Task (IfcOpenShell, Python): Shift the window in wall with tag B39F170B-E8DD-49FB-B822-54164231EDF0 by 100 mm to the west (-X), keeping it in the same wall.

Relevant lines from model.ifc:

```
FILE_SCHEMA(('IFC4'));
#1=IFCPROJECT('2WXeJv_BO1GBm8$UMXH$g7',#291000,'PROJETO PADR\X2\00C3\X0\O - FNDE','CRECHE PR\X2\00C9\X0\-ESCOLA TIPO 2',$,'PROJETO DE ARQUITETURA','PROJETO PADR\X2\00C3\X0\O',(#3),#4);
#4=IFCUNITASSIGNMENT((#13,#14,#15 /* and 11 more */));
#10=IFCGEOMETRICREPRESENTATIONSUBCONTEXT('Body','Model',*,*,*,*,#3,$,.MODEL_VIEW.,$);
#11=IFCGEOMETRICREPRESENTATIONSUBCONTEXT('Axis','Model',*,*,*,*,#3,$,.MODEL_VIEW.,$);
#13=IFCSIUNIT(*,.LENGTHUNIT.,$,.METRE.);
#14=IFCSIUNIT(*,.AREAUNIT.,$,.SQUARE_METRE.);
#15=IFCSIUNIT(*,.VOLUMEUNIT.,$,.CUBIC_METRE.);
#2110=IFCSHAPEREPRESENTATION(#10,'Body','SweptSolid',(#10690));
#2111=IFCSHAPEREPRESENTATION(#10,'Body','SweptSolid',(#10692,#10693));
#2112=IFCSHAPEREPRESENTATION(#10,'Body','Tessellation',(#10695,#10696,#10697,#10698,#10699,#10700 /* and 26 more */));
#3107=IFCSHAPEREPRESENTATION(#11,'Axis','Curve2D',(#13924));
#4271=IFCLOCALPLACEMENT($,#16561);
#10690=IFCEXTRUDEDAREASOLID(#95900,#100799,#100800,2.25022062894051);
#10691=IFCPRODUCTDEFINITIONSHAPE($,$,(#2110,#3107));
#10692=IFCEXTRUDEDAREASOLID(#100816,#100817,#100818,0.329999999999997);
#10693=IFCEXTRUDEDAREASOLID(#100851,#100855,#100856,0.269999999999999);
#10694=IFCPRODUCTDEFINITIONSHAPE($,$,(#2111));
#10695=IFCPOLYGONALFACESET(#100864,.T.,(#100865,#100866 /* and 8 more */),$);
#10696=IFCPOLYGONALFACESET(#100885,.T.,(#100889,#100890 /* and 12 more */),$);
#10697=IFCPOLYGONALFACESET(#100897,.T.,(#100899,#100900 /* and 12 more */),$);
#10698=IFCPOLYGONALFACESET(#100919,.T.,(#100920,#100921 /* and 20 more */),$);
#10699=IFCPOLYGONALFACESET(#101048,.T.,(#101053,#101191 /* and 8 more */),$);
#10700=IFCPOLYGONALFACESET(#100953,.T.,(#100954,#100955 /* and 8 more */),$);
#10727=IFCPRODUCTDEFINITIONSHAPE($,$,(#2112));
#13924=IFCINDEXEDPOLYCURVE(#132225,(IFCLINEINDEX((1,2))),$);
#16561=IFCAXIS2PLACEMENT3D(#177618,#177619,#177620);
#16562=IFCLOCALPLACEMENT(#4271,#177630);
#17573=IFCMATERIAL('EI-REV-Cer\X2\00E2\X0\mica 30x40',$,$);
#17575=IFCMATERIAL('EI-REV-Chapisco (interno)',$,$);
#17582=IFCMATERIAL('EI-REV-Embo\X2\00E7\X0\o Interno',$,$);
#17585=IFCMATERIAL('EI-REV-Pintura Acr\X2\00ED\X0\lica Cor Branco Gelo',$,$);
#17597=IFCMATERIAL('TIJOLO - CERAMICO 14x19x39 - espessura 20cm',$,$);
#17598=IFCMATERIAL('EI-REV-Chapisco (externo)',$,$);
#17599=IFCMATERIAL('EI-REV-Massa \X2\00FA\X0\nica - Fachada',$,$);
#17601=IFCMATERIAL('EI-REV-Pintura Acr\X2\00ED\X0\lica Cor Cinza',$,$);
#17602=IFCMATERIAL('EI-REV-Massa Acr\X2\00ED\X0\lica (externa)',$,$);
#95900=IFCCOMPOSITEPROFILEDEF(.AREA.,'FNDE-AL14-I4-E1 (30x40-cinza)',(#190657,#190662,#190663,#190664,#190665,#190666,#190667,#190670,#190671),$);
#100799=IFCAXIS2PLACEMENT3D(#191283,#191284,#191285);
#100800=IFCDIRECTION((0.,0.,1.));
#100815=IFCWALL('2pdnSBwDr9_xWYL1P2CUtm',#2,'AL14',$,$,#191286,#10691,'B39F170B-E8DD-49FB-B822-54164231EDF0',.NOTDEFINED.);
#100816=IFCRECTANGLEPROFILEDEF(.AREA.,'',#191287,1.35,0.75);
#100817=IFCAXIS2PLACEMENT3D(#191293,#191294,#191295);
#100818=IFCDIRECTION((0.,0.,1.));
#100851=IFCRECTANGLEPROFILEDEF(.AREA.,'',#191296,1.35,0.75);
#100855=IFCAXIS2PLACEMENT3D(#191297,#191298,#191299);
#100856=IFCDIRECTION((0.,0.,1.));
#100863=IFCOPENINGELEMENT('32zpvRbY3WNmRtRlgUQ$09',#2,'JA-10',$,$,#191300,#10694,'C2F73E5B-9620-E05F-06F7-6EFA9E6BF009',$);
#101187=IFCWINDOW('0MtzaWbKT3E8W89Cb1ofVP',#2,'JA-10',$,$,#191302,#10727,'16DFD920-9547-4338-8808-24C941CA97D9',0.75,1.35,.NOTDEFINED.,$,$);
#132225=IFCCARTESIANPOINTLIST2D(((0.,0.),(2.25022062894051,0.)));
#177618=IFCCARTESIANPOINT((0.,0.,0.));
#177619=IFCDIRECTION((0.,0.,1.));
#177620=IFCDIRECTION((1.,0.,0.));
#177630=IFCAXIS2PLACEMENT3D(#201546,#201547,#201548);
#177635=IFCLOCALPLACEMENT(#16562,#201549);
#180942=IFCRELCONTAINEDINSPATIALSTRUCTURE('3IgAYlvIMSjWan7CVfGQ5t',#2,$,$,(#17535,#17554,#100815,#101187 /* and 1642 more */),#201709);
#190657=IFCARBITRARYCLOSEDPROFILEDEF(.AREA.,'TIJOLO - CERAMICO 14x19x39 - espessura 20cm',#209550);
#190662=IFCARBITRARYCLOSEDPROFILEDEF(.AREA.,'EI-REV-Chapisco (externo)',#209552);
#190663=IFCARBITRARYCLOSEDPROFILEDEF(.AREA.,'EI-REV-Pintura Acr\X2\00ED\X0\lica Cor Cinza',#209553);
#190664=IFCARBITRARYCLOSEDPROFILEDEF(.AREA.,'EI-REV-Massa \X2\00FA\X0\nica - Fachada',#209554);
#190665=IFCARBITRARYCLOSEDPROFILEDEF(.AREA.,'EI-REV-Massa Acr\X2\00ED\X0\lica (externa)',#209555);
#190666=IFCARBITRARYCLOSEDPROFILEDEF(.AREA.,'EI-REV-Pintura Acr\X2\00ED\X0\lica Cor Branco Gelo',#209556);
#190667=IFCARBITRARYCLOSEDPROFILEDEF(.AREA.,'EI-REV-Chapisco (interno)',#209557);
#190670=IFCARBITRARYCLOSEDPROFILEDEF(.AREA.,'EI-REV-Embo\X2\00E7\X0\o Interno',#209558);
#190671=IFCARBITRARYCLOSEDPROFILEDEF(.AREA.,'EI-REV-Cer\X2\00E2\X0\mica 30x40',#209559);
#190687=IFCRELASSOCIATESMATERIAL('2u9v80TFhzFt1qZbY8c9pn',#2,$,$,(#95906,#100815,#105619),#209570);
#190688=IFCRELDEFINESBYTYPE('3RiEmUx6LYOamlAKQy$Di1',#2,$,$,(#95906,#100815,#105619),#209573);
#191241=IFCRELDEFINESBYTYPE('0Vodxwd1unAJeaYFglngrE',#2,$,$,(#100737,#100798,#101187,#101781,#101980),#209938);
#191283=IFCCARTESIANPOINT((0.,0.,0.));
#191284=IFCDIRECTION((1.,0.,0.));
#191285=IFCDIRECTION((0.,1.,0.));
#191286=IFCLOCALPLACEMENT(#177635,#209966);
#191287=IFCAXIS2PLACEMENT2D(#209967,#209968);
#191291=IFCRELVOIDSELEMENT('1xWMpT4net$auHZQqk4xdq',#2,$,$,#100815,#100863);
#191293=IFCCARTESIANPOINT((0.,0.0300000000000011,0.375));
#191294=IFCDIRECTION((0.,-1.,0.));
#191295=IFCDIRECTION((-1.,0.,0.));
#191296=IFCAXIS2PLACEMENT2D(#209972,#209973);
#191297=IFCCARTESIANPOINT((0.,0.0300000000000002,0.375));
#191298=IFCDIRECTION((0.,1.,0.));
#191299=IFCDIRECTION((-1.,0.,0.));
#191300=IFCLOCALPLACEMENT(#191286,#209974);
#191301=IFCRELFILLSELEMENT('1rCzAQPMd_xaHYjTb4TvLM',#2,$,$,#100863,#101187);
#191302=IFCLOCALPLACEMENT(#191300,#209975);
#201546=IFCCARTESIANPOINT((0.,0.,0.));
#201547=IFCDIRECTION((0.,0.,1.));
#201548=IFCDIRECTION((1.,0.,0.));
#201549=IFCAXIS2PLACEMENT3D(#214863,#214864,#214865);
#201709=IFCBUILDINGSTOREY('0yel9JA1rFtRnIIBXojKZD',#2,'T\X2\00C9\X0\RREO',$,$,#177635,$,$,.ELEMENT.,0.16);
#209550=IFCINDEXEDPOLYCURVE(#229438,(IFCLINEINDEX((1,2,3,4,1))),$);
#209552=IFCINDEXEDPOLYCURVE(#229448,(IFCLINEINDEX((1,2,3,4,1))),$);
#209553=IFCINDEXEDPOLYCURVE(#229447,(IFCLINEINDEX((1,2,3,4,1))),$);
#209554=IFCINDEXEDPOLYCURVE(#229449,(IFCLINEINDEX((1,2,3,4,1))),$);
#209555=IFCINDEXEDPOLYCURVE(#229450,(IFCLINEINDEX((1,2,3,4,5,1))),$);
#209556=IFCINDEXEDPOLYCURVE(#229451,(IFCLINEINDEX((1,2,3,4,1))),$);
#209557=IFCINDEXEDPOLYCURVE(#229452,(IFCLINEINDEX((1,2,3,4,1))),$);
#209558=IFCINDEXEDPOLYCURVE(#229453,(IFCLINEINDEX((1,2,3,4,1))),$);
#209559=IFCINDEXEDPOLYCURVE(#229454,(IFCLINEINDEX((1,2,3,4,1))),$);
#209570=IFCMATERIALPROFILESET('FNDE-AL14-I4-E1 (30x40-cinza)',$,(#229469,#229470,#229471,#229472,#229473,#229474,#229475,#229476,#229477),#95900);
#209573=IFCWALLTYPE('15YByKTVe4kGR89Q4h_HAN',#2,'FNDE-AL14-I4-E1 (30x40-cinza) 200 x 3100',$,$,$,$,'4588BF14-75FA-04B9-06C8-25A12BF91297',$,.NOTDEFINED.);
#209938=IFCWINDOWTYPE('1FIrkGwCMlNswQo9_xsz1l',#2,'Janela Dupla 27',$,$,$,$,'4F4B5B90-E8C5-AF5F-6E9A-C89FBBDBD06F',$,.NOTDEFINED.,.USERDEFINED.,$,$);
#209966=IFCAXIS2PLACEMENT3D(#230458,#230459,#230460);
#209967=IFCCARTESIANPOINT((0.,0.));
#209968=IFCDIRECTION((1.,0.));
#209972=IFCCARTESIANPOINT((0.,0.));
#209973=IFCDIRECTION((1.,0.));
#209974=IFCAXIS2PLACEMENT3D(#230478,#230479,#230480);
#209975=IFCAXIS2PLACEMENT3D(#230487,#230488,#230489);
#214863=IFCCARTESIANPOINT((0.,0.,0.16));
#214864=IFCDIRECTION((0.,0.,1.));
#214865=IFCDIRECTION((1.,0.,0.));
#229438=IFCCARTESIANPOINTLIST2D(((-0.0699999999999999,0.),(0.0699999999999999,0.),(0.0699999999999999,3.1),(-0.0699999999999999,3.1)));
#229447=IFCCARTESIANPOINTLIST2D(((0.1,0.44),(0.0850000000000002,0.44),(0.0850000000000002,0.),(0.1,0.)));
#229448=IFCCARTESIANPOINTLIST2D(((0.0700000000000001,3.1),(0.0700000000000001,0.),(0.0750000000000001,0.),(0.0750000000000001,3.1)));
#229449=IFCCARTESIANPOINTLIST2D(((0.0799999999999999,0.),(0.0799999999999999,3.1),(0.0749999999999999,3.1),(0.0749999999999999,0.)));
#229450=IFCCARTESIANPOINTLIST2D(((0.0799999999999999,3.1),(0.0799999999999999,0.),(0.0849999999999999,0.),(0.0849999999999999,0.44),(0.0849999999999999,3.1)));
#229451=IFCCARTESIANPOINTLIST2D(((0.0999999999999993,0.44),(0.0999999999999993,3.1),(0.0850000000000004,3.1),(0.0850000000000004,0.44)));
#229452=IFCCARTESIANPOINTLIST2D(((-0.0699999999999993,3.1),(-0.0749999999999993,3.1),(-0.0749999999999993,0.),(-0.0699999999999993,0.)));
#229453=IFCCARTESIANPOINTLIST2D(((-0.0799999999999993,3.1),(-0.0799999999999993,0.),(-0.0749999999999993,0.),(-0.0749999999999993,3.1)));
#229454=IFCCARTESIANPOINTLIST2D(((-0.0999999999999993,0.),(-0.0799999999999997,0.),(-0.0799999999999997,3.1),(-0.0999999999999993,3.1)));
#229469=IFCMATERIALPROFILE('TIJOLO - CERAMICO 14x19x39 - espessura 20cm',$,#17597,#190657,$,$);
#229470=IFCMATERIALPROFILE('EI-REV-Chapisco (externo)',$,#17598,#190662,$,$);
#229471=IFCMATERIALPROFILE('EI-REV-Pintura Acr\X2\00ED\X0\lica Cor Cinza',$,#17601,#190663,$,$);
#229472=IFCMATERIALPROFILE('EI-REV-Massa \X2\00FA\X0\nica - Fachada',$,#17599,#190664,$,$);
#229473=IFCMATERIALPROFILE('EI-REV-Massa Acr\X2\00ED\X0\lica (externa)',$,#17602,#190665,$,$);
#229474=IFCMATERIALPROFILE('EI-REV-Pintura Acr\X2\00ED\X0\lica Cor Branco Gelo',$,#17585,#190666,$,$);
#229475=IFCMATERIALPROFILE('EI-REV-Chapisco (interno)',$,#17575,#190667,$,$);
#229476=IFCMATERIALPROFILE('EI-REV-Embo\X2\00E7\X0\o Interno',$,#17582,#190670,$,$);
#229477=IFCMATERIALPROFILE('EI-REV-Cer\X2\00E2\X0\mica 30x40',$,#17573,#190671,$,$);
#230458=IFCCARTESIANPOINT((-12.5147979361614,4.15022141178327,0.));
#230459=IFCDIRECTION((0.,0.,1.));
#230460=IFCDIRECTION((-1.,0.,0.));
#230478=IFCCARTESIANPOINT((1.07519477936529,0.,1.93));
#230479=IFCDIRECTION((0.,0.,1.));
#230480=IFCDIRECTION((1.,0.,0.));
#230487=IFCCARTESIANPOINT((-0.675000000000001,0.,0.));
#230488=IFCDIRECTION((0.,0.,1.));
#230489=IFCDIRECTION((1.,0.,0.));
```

```python
import ifcopenshell
import ifcopenshell.api.geometry
import ifcopenshell.util.placement

model = ifcopenshell.open("model.ifc")

window = model.by_guid("0MtzaWbKT3E8W89Cb1ofVP")
opening = window.FillsVoids[0].RelatingOpeningElement
wall = opening.VoidsElements[0].RelatingBuildingElement

wall_matrix = ifcopenshell.util.placement.get_local_placement(wall.ObjectPlacement)
shift = wall_matrix[:3, 0] * 0.1
before = ifcopenshell.util.placement.get_local_placement(window.ObjectPlacement)[:3, 3].copy()

# The window is placed relative to its opening, so it follows when the opening moves.
matrix = ifcopenshell.util.placement.get_local_placement(opening.ObjectPlacement)
matrix[:3, 3] += shift
ifcopenshell.api.geometry.edit_object_placement(
    model, product=opening, matrix=matrix, is_si=False, should_transform_children=True
)

after = ifcopenshell.util.placement.get_local_placement(window.ObjectPlacement)[:3, 3]
print("window moved by", (after - before).round(3) + 0.0)

model.write("model_rev.ifc")
```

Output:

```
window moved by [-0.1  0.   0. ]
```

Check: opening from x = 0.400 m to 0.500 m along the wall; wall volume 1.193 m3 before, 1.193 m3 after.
